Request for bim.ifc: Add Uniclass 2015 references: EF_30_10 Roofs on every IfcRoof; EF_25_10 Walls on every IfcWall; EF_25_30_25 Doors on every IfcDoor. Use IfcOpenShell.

First a look at what the model holds.

```python
import ifcopenshell

model = ifcopenshell.open("bim.ifc")
print(model.schema)
print("classifications:", [c.Name for c in model.by_type("IfcClassification")])
for ifc_class in ("IfcDoor", "IfcRoof", "IfcStair", "IfcWall", "IfcWindow"):
    print(ifc_class, len(model.by_type(ifc_class)))
```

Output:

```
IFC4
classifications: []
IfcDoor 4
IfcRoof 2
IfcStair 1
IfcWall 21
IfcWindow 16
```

```python
import ifcopenshell
import ifcopenshell.api.classification

model = ifcopenshell.open("bim.ifc")

system = ifcopenshell.api.classification.add_classification(model, classification="Uniclass 2015")

codes = {
    "IfcRoof": ("EF_30_10", "Roofs"),
    "IfcWall": ("EF_25_10", "Walls"),
    "IfcDoor": ("EF_25_30_25", "Doors"),
}
for ifc_class, (code, name) in codes.items():
    products = model.by_type(ifc_class)
    ifcopenshell.api.classification.add_reference(
        model, products=products, classification=system, identification=code, name=name
    )
    print(code, len(products))

model.write("bim-out.ifc")
```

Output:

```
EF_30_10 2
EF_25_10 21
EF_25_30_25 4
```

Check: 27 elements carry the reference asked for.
